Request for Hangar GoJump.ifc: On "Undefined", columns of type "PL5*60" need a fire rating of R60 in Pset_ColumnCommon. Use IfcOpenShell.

First a look at what the model holds.

```python
import ifcopenshell
import ifcopenshell.util.element

model = ifcopenshell.open("Hangar GoJump.ifc")
print(model.schema)
storey = next(s for s in model.by_type("IfcBuildingStorey") if s.Name == "Undefined")
columns = [e for e in ifcopenshell.util.element.get_decomposition(storey) if e.is_a("IfcColumn")]
seen = {}
for e in columns:
    element_type = ifcopenshell.util.element.get_type(e)
    key = (element_type.Name if element_type != e and element_type else None, ifcopenshell.util.element.get_pset(e, "Pset_ColumnCommon", "FireRating"))
    seen[key] = seen.get(key, 0) + 1
for (name, value), count in sorted(seen.items(), key=str):
    print(count, "x", name, "|", value)
```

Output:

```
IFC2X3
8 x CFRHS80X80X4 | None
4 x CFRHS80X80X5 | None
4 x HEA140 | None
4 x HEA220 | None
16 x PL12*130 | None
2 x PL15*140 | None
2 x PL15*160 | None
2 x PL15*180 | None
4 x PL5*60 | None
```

```python
import ifcopenshell
import ifcopenshell.api.pset
import ifcopenshell.util.element

model = ifcopenshell.open("Hangar GoJump.ifc")

storey = next(s for s in model.by_type("IfcBuildingStorey") if s.Name == "Undefined")
columns = [e for e in ifcopenshell.util.element.get_decomposition(storey) if e.is_a("IfcColumn")]

count = 0
for e in columns:
    element_type = ifcopenshell.util.element.get_type(e)
    if element_type in (None, e) or element_type.Name != "PL5*60":
        continue
    # add_pset returns the element's existing set when there is one.
    pset = ifcopenshell.api.pset.add_pset(model, product=e, name="Pset_ColumnCommon")
    ifcopenshell.api.pset.edit_pset(model, pset=pset, properties={"FireRating": "R60"})
    count += 1

print(count, "columns updated")

model.write("Hangar GoJump_v2.ifc")
```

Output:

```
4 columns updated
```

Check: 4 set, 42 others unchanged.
